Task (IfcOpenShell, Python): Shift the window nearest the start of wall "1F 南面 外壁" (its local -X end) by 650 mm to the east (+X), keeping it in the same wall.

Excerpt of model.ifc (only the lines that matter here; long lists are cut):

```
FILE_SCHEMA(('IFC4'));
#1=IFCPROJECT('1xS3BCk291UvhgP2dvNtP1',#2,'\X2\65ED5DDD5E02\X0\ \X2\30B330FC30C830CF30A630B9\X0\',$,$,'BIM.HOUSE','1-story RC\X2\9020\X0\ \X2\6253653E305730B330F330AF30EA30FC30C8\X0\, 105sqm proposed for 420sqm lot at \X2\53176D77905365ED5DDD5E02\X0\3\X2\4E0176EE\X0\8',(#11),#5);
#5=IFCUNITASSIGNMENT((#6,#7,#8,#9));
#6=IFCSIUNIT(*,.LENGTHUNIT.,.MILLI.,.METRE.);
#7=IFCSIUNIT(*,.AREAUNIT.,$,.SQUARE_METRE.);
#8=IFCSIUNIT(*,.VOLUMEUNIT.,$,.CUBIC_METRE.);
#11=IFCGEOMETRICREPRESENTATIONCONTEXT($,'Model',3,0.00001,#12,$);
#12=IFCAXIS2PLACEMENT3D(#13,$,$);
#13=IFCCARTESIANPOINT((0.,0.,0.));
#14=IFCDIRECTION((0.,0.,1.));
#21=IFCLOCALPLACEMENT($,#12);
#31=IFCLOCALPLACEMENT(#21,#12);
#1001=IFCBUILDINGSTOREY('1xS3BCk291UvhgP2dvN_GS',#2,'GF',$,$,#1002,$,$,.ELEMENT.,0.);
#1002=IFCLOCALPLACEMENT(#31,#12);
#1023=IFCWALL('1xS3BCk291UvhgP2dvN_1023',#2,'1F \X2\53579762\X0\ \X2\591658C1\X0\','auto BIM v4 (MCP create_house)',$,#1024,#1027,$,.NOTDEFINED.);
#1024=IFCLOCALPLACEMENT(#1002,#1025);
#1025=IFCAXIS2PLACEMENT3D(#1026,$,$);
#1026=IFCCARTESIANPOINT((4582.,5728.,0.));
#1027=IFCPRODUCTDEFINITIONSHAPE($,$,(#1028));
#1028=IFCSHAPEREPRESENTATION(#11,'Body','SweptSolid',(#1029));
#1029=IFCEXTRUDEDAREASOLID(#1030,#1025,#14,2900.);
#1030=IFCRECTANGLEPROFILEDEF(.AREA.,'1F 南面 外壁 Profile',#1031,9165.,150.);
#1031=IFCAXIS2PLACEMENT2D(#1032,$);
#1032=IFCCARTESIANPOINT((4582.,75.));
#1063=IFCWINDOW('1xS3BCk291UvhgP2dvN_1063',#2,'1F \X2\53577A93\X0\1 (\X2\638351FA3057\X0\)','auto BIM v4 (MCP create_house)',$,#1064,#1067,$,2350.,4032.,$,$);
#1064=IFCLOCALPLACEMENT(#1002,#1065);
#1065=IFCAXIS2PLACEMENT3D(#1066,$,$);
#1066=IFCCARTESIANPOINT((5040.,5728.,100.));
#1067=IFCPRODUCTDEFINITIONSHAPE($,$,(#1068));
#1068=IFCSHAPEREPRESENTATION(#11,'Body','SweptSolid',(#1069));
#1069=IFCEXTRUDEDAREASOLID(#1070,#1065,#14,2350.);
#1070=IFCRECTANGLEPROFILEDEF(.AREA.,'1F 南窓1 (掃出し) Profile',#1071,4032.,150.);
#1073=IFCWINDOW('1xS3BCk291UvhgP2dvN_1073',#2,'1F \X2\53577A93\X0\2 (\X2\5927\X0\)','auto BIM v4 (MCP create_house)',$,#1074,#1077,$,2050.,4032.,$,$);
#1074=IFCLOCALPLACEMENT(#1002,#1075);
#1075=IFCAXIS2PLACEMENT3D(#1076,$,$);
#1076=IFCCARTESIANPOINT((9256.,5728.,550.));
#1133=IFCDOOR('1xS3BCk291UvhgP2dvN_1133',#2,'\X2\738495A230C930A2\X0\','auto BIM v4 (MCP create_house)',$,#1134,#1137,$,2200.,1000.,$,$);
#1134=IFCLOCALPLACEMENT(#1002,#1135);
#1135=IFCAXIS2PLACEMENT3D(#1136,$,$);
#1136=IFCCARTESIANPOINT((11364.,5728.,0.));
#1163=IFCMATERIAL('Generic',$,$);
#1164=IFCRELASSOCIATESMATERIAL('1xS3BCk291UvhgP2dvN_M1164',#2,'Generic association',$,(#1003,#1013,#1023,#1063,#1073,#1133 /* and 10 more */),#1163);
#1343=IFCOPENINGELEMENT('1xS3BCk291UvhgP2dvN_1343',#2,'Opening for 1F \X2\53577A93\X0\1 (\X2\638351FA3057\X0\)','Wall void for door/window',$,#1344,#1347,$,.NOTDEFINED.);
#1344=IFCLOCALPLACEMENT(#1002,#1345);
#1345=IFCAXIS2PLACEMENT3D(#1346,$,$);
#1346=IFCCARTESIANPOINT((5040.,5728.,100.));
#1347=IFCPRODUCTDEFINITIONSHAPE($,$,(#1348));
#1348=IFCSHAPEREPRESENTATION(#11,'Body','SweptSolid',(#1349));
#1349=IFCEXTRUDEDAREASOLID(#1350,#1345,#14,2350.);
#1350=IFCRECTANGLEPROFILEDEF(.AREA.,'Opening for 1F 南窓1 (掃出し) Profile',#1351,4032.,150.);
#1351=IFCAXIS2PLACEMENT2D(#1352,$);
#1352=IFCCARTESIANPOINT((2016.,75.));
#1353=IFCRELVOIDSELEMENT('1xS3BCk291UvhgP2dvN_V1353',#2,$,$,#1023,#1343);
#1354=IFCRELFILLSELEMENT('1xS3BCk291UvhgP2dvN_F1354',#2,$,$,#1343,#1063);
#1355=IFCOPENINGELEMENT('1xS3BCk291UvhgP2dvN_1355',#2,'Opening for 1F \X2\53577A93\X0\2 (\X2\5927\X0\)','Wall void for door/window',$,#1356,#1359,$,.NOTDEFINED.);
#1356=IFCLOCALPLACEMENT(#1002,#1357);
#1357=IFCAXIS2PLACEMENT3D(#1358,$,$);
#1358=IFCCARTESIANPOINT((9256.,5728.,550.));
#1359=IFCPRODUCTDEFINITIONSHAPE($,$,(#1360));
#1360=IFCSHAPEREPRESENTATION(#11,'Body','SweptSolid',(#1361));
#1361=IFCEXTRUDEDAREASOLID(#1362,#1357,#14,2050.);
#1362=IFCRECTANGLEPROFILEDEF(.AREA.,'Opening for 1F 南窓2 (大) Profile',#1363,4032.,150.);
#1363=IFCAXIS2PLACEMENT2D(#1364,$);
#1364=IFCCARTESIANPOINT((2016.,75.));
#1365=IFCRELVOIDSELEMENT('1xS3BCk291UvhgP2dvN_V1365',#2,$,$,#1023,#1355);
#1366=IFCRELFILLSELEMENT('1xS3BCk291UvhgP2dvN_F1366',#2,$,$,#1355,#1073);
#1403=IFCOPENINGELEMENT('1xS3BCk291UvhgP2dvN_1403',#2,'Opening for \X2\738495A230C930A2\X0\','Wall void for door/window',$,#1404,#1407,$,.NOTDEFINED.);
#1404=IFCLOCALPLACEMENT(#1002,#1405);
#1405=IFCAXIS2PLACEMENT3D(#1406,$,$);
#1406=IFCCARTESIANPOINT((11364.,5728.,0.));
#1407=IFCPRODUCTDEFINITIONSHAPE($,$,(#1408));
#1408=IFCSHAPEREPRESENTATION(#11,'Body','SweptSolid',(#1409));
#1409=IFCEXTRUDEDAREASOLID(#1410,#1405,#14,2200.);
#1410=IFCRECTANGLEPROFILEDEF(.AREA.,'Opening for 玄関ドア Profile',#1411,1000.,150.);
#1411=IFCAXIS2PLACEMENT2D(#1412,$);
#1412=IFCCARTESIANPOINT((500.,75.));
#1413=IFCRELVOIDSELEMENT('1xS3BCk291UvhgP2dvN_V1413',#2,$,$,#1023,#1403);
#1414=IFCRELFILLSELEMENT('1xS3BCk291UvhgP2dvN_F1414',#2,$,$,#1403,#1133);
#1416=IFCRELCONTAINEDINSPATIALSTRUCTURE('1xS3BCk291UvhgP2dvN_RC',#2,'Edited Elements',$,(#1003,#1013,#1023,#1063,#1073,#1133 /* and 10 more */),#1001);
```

```python
import ifcopenshell
import ifcopenshell.api.geometry
import ifcopenshell.util.placement
import ifcopenshell.util.unit

model = ifcopenshell.open("model.ifc")
unit_scale = ifcopenshell.util.unit.calculate_unit_scale(model)

window = model.by_id(1063)
opening = window.FillsVoids[0].RelatingOpeningElement
wall = opening.VoidsElements[0].RelatingBuildingElement

wall_matrix = ifcopenshell.util.placement.get_local_placement(wall.ObjectPlacement)
shift = wall_matrix[:3, 0] * 0.65 / unit_scale
before = ifcopenshell.util.placement.get_local_placement(window.ObjectPlacement)[:3, 3].copy()

# The window is not placed relative to its opening, so move both.
for product in (opening, window):
    matrix = ifcopenshell.util.placement.get_local_placement(product.ObjectPlacement)
    matrix[:3, 3] += shift
    ifcopenshell.api.geometry.edit_object_placement(model, product=product, matrix=matrix, is_si=False)

after = ifcopenshell.util.placement.get_local_placement(window.ObjectPlacement)[:3, 3]
print("window moved by", (after - before).round(3) + 0.0)

model.write("model-out.ifc")
```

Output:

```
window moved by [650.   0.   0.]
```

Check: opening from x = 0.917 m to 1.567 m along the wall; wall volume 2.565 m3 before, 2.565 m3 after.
